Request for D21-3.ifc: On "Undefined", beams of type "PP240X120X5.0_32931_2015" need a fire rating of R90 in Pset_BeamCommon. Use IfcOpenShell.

First a look at what the model holds.

```python
import ifcopenshell
import ifcopenshell.util.element

model = ifcopenshell.open("D21-3.ifc")
print(model.schema)
storey = next(s for s in model.by_type("IfcBuildingStorey") if s.Name == "Undefined")
beams = [e for e in ifcopenshell.util.element.get_decomposition(storey) if e.is_a("IfcBeam")]
seen = {}
for e in beams:
    element_type = ifcopenshell.util.element.get_type(e)
    key = (element_type.Name if element_type != e and element_type else None, ifcopenshell.util.element.get_pset(e, "Pset_BeamCommon", "FireRating"))
    seen[key] = seen.get(key, 0) + 1
for (name, value), count in sorted(seen.items(), key=str):
    print(count, "x", name, "|", value)
```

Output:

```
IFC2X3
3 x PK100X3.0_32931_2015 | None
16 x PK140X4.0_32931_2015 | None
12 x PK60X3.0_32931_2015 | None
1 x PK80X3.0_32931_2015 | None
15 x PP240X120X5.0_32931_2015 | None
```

```python
import ifcopenshell
import ifcopenshell.api.pset
import ifcopenshell.util.element

model = ifcopenshell.open("D21-3.ifc")

storey = next(s for s in model.by_type("IfcBuildingStorey") if s.Name == "Undefined")
beams = [e for e in ifcopenshell.util.element.get_decomposition(storey) if e.is_a("IfcBeam")]

count = 0
for e in beams:
    element_type = ifcopenshell.util.element.get_type(e)
    if element_type in (None, e) or element_type.Name != "PP240X120X5.0_32931_2015":
        continue
    found = ifcopenshell.util.element.get_pset(e, "Pset_BeamCommon", should_inherit=False)
    if found:
        pset = model.by_id(found["id"])
        if len(ifcopenshell.util.element.get_elements_by_pset(pset)) > 1:
            pset = ifcopenshell.api.pset.unshare_pset(model, products=[e], pset=pset)[0]
    else:
        pset = ifcopenshell.api.pset.add_pset(model, product=e, name="Pset_BeamCommon")
    ifcopenshell.api.pset.edit_pset(model, pset=pset, properties={"FireRating": "R90"})
    count += 1

print(count, "beams updated")

model.write("D21-3_updated.ifc")
```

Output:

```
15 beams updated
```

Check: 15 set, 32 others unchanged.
